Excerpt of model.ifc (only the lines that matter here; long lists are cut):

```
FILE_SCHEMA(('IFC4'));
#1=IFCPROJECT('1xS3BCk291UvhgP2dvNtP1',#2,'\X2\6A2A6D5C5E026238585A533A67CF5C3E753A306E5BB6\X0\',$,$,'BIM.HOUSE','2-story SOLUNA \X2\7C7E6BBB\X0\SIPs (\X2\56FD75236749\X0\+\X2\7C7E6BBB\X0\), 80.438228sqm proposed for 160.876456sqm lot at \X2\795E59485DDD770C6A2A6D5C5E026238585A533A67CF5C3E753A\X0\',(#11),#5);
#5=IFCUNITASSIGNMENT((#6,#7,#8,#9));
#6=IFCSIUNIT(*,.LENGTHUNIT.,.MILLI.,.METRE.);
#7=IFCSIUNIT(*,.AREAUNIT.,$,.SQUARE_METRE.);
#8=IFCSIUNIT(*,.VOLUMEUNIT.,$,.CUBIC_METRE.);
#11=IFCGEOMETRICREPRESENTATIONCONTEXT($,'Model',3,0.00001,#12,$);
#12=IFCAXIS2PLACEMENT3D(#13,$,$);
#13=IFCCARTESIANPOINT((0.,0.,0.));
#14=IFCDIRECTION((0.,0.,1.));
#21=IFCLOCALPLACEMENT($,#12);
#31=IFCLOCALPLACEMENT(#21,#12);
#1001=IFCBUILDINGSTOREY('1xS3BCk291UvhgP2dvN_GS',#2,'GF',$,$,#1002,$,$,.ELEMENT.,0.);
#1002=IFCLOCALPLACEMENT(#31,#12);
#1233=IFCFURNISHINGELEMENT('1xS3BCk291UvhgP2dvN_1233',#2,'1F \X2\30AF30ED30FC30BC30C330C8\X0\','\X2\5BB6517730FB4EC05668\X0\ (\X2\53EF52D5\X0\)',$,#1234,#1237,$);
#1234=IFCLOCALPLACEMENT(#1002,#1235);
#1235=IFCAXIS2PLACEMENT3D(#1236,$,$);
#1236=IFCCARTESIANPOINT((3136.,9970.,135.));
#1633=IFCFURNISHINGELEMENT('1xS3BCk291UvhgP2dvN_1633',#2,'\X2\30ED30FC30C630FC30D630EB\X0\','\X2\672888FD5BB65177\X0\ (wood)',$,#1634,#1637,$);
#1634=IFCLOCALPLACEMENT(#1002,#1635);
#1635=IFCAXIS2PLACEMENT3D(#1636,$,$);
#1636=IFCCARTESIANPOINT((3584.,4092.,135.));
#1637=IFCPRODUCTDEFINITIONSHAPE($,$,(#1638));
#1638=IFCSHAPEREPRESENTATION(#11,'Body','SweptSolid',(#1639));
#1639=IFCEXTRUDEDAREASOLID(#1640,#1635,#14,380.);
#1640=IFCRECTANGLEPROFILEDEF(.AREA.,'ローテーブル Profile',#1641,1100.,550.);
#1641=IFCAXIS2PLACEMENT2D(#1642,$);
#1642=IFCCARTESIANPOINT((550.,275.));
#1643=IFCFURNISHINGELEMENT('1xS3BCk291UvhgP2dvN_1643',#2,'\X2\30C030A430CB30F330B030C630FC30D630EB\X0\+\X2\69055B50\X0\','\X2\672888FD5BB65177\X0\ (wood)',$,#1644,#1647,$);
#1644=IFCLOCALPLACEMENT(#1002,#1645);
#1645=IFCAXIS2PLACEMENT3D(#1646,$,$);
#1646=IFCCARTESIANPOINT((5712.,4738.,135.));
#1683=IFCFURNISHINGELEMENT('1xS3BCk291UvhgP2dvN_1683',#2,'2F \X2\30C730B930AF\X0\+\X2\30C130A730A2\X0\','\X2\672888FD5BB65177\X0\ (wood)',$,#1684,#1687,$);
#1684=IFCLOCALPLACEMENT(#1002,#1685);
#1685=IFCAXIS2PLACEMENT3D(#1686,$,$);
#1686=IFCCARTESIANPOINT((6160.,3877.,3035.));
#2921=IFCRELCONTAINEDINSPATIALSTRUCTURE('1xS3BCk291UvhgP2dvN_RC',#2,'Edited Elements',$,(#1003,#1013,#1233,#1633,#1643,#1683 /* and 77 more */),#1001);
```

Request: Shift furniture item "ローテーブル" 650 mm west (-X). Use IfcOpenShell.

```python
import ifcopenshell
import ifcopenshell.api.geometry
import ifcopenshell.util.placement
import ifcopenshell.util.unit

model = ifcopenshell.open("model.ifc")
unit_scale = ifcopenshell.util.unit.calculate_unit_scale(model)

item = model.by_guid("1xS3BCk291UvhgP2dvN_1633")
matrix = ifcopenshell.util.placement.get_local_placement(item.ObjectPlacement)
matrix[0, 3] -= 0.65 / unit_scale
ifcopenshell.api.geometry.edit_object_placement(model, product=item, matrix=matrix, is_si=False)

print(ifcopenshell.util.placement.get_local_placement(item.ObjectPlacement).round(3) + 0.0)

model.write("model-out.ifc")
```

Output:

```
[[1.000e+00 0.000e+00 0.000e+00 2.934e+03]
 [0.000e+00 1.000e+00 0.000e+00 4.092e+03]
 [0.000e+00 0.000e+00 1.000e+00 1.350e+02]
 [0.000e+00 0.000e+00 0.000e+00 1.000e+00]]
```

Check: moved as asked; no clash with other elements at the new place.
